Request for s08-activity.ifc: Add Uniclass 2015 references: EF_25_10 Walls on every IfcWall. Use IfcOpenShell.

First a look at what the model holds.

```python
import ifcopenshell

model = ifcopenshell.open("s08-activity.ifc")
print(model.schema)
print("classifications:", [c.Name for c in model.by_type("IfcClassification")])
for ifc_class in ("IfcDoor", "IfcRoof", "IfcStair", "IfcWall", "IfcWindow"):
    print(ifc_class, len(model.by_type(ifc_class)))
```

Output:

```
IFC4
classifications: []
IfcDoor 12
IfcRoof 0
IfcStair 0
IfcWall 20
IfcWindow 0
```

```python
import ifcopenshell
import ifcopenshell.api.classification

model = ifcopenshell.open("s08-activity.ifc")

system = ifcopenshell.api.classification.add_classification(model, classification="Uniclass 2015")

codes = {
    "IfcWall": ("EF_25_10", "Walls"),
}
for ifc_class, (code, name) in codes.items():
    products = model.by_type(ifc_class)
    ifcopenshell.api.classification.add_reference(
        model, products=products, classification=system, identification=code, name=name
    )
    print(code, len(products))

model.write("s08-activity_updated.ifc")
```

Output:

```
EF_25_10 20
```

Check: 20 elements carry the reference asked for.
